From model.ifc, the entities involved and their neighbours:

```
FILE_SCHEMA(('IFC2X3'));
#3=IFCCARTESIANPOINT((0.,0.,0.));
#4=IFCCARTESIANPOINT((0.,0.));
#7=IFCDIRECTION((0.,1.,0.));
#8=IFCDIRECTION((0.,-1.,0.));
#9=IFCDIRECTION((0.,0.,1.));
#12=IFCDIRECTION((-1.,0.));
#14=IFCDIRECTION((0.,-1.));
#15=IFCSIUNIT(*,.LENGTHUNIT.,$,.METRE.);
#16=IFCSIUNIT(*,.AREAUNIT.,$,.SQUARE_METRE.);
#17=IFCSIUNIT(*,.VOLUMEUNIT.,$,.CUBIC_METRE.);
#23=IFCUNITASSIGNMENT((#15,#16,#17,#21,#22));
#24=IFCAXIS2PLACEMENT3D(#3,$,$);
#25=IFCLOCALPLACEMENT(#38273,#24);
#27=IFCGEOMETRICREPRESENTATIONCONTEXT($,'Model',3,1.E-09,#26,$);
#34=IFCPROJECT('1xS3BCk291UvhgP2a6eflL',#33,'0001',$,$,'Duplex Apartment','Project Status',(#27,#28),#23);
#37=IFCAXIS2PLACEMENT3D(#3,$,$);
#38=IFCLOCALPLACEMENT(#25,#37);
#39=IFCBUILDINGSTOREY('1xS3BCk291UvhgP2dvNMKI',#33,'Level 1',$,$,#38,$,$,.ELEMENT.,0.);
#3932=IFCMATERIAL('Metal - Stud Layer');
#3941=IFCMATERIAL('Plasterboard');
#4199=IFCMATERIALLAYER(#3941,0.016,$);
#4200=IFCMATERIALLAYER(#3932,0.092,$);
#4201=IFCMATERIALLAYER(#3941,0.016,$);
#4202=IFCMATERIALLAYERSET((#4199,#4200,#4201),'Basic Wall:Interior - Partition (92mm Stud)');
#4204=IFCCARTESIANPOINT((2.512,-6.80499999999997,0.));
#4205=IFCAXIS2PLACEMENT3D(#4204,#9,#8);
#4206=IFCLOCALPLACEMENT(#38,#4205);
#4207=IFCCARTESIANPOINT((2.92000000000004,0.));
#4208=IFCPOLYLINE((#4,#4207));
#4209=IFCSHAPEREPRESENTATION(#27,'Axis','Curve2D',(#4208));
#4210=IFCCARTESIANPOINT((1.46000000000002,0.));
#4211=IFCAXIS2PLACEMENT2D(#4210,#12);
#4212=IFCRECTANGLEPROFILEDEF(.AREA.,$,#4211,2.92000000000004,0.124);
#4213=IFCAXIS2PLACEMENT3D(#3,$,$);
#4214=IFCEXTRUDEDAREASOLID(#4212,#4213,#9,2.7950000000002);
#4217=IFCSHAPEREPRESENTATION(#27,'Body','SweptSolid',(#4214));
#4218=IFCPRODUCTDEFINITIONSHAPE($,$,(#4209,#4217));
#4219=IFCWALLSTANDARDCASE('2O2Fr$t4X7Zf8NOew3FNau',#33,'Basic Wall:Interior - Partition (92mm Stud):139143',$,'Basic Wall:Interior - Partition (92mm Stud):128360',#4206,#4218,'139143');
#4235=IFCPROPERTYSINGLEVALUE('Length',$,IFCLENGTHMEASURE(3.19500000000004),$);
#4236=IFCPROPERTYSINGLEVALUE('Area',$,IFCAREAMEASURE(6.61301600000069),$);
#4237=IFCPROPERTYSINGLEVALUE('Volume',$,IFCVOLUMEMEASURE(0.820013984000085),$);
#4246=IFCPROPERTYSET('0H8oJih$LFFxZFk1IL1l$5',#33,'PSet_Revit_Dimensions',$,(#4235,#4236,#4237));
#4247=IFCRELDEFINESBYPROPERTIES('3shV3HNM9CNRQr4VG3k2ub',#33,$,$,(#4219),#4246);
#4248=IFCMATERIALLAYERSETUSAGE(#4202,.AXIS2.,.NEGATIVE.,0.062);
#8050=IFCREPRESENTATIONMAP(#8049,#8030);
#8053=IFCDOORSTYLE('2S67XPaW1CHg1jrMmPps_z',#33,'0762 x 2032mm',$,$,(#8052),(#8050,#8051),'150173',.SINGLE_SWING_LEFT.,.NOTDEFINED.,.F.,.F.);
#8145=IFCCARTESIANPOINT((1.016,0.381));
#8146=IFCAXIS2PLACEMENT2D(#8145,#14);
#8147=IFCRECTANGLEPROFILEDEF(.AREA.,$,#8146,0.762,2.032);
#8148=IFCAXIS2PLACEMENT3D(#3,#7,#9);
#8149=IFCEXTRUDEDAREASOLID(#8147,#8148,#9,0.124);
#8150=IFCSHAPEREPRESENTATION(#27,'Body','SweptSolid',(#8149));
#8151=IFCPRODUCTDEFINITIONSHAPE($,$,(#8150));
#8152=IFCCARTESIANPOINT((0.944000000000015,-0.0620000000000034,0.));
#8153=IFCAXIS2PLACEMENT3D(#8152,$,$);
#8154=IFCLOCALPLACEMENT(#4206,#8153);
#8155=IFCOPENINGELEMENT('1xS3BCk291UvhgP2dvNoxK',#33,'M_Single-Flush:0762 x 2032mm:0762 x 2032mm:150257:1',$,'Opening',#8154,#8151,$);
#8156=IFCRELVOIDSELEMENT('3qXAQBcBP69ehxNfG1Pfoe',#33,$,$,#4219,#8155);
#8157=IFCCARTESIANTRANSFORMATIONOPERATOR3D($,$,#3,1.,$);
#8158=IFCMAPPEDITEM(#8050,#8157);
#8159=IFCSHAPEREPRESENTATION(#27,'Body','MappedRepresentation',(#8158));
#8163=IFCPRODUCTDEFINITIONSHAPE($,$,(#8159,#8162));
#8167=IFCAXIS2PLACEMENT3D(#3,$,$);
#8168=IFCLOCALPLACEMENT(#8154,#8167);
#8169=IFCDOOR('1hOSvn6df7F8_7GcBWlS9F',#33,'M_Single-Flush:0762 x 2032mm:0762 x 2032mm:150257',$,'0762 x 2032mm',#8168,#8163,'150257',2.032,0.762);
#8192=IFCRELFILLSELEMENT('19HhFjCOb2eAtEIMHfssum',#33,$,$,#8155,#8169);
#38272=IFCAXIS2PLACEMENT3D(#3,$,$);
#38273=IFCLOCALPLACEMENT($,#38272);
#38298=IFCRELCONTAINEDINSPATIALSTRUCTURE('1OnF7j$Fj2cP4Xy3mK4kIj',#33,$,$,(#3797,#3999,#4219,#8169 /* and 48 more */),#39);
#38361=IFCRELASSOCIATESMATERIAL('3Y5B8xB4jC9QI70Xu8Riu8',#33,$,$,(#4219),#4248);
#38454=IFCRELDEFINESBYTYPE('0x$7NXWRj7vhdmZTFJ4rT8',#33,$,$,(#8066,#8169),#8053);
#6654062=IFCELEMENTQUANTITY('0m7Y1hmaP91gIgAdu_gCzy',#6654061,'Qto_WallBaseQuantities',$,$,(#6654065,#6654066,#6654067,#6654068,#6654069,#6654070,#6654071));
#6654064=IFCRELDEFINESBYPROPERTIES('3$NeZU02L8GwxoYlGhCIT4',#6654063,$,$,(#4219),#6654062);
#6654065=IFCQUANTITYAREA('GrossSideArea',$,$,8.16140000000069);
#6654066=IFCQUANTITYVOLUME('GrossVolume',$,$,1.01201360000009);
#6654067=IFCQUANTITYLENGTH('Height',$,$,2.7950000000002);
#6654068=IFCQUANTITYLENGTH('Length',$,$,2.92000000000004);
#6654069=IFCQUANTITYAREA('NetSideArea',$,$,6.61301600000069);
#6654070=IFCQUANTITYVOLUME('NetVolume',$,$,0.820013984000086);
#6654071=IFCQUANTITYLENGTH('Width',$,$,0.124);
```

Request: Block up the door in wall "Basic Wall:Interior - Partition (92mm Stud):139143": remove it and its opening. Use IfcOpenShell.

```python
import ifcopenshell
import ifcopenshell.api.feature
import ifcopenshell.api.pset
import ifcopenshell.api.root
import ifcopenshell.geom
import ifcopenshell.util.element
import ifcopenshell.util.shape
import ifcopenshell.util.unit

model = ifcopenshell.open("model.ifc")
area_scale = ifcopenshell.util.unit.calculate_unit_scale(model, "AREAUNIT")
volume_scale = ifcopenshell.util.unit.calculate_unit_scale(model, "VOLUMEUNIT")
settings = ifcopenshell.geom.settings()


def volume(element):
    """Net volume in cubic metres, openings subtracted."""
    shape = ifcopenshell.geom.create_shape(settings, element)
    return ifcopenshell.util.shape.get_volume(shape.geometry)


door = model.by_id(8169)
opening = door.FillsVoids[0].RelatingOpeningElement
wall = opening.VoidsElements[0].RelatingBuildingElement
before = volume(wall)

ifcopenshell.api.root.remove_product(model, product=door)
ifcopenshell.api.feature.remove_feature(model, feature=opening)

after = volume(wall)
thickness = 0.124  # wall thickness in metres

# Update the wall's stored quantities.
pset = model.by_id(ifcopenshell.util.element.get_pset(wall, "PSet_Revit_Dimensions", should_inherit=False)["id"])
ifcopenshell.api.pset.edit_pset(model, pset=pset, properties={
    "Area": model.create_entity("IfcAreaMeasure", after / thickness / area_scale),
    "Volume": model.create_entity("IfcVolumeMeasure", after / volume_scale),
})
qto = model.by_id(ifcopenshell.util.element.get_pset(wall, "Qto_WallBaseQuantities", should_inherit=False)["id"])
ifcopenshell.api.pset.edit_qto(model, qto=qto, properties={
    "NetSideArea": after / thickness / area_scale,
    "NetVolume": after / volume_scale,
})

print(f"wall volume {before:.3f} -> {after:.3f} m3")

model.write("model_v2.ifc")
```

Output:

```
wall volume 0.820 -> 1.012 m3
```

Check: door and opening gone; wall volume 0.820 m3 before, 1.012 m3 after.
